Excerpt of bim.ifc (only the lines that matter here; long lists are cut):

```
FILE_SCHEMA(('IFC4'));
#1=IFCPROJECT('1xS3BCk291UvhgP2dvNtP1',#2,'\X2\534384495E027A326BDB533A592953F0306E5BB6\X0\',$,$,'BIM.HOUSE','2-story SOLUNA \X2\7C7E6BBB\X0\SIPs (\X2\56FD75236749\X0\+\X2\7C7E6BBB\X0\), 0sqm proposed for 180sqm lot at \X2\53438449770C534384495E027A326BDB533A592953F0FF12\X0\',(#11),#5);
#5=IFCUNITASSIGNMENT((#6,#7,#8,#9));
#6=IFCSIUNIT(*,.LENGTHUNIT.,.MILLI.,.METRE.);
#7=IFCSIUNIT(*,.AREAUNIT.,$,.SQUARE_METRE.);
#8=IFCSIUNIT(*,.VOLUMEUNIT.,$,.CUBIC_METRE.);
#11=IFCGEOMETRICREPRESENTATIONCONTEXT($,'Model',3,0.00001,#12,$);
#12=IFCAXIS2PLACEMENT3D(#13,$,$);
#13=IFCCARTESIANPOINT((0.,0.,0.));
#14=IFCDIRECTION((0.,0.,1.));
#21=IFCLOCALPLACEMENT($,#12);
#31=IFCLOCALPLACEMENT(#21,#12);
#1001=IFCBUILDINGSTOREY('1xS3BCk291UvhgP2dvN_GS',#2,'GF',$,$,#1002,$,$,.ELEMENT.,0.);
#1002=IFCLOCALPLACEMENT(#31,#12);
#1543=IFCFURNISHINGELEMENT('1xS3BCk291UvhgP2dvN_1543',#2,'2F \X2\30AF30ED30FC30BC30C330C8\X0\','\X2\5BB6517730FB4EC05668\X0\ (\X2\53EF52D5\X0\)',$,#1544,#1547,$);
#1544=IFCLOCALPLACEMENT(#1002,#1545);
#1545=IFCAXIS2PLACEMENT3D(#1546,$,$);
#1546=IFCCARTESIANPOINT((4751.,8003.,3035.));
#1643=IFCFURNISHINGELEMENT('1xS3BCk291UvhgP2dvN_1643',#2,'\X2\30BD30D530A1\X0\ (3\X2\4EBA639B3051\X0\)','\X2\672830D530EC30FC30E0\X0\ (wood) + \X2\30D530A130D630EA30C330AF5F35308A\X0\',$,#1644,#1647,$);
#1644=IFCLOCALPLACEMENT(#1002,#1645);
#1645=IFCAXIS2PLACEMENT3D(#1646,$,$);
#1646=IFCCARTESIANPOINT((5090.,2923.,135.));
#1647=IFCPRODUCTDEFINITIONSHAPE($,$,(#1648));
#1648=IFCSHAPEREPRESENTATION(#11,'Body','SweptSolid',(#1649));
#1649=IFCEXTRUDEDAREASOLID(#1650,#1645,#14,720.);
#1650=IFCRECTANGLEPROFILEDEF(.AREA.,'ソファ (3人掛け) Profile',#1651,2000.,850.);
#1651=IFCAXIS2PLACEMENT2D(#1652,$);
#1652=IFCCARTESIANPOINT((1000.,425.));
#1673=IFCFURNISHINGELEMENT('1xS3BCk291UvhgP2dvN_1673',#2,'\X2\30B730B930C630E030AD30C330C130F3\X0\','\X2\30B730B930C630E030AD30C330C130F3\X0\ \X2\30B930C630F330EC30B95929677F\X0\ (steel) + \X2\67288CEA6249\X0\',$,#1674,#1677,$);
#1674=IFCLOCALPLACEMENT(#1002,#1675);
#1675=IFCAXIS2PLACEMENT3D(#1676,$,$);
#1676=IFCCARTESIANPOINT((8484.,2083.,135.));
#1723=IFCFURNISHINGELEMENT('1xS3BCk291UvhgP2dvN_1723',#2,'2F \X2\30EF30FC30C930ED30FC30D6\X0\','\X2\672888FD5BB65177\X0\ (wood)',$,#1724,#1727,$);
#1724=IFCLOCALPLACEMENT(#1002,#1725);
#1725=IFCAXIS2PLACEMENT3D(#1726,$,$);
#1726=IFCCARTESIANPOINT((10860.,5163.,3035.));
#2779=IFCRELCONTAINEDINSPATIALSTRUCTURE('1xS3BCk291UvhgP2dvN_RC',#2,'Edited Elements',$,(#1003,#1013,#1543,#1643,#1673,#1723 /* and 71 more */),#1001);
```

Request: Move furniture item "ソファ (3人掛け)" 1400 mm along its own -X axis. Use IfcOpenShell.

```python
import ifcopenshell
import ifcopenshell.api.geometry
import ifcopenshell.util.placement

model = ifcopenshell.open("bim.ifc")

item = model.by_guid("1xS3BCk291UvhgP2dvN_1643")
matrix = ifcopenshell.util.placement.get_local_placement(item.ObjectPlacement)
matrix[:3, 3] -= matrix[:3, 0] * 1400.0
ifcopenshell.api.geometry.edit_object_placement(model, product=item, matrix=matrix, is_si=False)

print(ifcopenshell.util.placement.get_local_placement(item.ObjectPlacement).round(3) + 0.0)

model.write("bim_rev.ifc")
```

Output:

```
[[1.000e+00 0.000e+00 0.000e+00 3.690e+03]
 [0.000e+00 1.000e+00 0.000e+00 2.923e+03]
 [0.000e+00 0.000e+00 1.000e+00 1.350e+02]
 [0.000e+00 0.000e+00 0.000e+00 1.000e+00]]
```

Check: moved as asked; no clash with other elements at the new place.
